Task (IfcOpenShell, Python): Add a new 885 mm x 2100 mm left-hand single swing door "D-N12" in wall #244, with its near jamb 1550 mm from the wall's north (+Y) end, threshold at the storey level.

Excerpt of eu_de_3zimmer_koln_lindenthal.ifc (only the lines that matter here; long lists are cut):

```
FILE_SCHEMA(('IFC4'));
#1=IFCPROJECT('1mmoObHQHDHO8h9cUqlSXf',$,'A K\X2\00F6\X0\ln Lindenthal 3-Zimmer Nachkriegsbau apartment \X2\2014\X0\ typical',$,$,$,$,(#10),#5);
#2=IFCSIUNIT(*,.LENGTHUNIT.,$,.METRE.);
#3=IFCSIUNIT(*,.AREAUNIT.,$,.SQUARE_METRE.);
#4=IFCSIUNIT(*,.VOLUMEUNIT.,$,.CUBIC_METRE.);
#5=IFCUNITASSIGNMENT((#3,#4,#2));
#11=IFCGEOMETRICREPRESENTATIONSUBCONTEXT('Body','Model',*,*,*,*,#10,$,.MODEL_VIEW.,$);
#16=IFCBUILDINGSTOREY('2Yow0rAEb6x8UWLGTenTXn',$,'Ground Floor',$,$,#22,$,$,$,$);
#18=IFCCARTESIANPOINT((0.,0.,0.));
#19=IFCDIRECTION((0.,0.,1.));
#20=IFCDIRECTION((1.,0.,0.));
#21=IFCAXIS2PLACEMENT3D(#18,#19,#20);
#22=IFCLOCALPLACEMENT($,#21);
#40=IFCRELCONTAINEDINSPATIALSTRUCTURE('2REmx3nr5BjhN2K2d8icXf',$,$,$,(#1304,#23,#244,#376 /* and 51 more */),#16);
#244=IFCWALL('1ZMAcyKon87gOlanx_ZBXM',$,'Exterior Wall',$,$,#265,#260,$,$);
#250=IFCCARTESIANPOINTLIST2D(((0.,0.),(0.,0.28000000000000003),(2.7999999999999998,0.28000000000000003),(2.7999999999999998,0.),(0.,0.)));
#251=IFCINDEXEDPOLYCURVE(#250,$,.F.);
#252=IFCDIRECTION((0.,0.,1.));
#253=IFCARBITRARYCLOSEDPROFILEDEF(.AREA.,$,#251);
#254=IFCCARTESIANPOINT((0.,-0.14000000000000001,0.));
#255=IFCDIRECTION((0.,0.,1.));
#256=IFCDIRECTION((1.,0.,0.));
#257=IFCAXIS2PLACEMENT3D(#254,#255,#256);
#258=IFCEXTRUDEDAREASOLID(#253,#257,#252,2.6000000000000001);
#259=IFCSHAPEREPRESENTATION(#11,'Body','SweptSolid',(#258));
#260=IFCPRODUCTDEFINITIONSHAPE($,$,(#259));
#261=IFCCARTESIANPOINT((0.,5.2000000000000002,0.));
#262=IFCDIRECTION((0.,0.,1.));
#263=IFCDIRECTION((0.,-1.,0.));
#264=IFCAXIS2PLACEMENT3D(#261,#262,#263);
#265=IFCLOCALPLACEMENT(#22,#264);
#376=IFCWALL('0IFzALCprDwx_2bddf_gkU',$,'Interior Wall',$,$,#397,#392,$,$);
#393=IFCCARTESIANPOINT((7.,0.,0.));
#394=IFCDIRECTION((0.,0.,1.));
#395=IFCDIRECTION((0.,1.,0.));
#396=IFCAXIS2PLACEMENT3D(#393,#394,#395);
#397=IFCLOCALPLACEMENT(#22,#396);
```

```python
import numpy as np
import ifcopenshell
import ifcopenshell.api.feature
import ifcopenshell.api.geometry
import ifcopenshell.api.root
import ifcopenshell.api.spatial
import ifcopenshell.geom
import ifcopenshell.util.element
import ifcopenshell.util.placement
import ifcopenshell.util.representation
import ifcopenshell.util.shape
import ifcopenshell.util.unit

model = ifcopenshell.open("eu_de_3zimmer_koln_lindenthal.ifc")
unit_scale = ifcopenshell.util.unit.calculate_unit_scale(model)
settings = ifcopenshell.geom.settings()


def volume(element):
    """Net volume in cubic metres, openings subtracted."""
    shape = ifcopenshell.geom.create_shape(settings, element)
    return ifcopenshell.util.shape.get_volume(shape.geometry)


wall = model.by_id(244)
storey = ifcopenshell.util.element.get_container(wall, ifc_class="IfcBuildingStorey")
context = ifcopenshell.util.representation.get_context(model, "Model", "Body", "MODEL_VIEW")
before = volume(wall)

width, height, from_end, sill = 0.885, 2.1, 1.55, 0.0  # metres

# The wall runs along its own X axis, and the end named is its -X end.
wall_shape = ifcopenshell.geom.create_shape(settings, wall)
x, y, z = ifcopenshell.util.shape.get_vertices(wall_shape.geometry).T
start = x.min() + from_end
face, thickness = float(y.min()), float(y.max() - y.min())
wall_matrix = ifcopenshell.util.placement.get_local_placement(wall.ObjectPlacement)
level = ifcopenshell.util.placement.get_local_placement(storey.ObjectPlacement)[2, 3]


def in_wall(x, y):
    """Placement at x, y metres in the wall's axes, at sill height."""
    matrix = wall_matrix.copy()
    matrix[:, 3] = wall_matrix @ np.array([x / unit_scale, y / unit_scale, 0.0, 1.0])
    matrix[2, 3] = level + sill / unit_scale
    return matrix


# Opening: a box that overshoots both wall faces by 50 mm.
opening = ifcopenshell.api.root.create_entity(model, ifc_class="IfcOpeningElement", predefined_type="OPENING")
box = ifcopenshell.api.geometry.add_wall_representation(
    model, context=context, length=width, height=height, thickness=thickness + 0.1
)
ifcopenshell.api.geometry.assign_representation(model, product=opening, representation=box)
ifcopenshell.api.geometry.edit_object_placement(model, product=opening, matrix=in_wall(start, face - 0.05), is_si=False)
ifcopenshell.api.feature.add_feature(model, feature=opening, element=wall)

door = ifcopenshell.api.root.create_entity(model, ifc_class="IfcDoor", name="D-N12", predefined_type="DOOR")
door.OverallWidth, door.OverallHeight = width / unit_scale, height / unit_scale
door.OperationType = "SINGLE_SWING_LEFT"
body = ifcopenshell.api.geometry.add_door_representation(
    model,
    context=context,
    overall_width=door.OverallWidth,
    overall_height=door.OverallHeight,
    operation_type="SINGLE_SWING_LEFT",
    lining_properties={"LiningDepth": thickness / unit_scale, "ThresholdDepth": thickness / unit_scale},
)
ifcopenshell.api.geometry.assign_representation(model, product=door, representation=body)
ifcopenshell.api.spatial.assign_container(model, products=[door], relating_structure=storey)
ifcopenshell.api.feature.add_filling(model, opening=opening, element=door)

# The lining spans the wall, so the door starts at the wall face.
ifcopenshell.api.geometry.edit_object_placement(model, product=door, matrix=in_wall(start, face), is_si=False)

after = volume(wall)

print(f"wall volume {before:.3f} -> {after:.3f} m3")

model.write("eu_de_3zimmer_koln_lindenthal-out.ifc")
```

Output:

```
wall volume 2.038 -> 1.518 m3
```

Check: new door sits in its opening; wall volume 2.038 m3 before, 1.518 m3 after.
